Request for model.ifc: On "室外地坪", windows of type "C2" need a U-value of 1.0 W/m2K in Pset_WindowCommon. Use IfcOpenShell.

First a look at what the model holds.

```python
import ifcopenshell
import ifcopenshell.util.element

model = ifcopenshell.open("model.ifc")
print(model.schema)
storey = next(s for s in model.by_type("IfcBuildingStorey") if s.Name == "室外地坪")
windows = [e for e in ifcopenshell.util.element.get_decomposition(storey) if e.is_a("IfcWindow")]
seen = {}
for e in windows:
    element_type = ifcopenshell.util.element.get_type(e)
    key = (element_type.Name if element_type != e and element_type else None, ifcopenshell.util.element.get_pset(e, "Pset_WindowCommon", "ThermalTransmittance"))
    seen[key] = seen.get(key, 0) + 1
for (name, value), count in sorted(seen.items(), key=str):
    print(count, "x", name, "|", value)
```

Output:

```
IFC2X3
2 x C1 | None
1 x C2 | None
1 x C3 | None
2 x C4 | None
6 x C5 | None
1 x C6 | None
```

```python
import ifcopenshell
import ifcopenshell.api.pset
import ifcopenshell.util.element

model = ifcopenshell.open("model.ifc")

storey = next(s for s in model.by_type("IfcBuildingStorey") if s.Name == "室外地坪")
windows = [e for e in ifcopenshell.util.element.get_decomposition(storey) if e.is_a("IfcWindow")]

count = 0
for e in windows:
    element_type = ifcopenshell.util.element.get_type(e)
    if element_type in (None, e) or element_type.Name != "C2":
        continue
    # add_pset returns the element's existing set when there is one.
    pset = ifcopenshell.api.pset.add_pset(model, product=e, name="Pset_WindowCommon")
    ifcopenshell.api.pset.edit_pset(model, pset=pset, properties={"ThermalTransmittance": 1.0})
    count += 1

print(count, "windows updated")

model.write("model_edited.ifc")
```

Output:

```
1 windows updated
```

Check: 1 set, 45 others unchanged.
